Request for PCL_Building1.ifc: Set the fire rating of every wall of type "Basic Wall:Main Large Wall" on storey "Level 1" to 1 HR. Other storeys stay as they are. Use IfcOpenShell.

First a look at what the model holds.

```python
import ifcopenshell
import ifcopenshell.util.element

model = ifcopenshell.open("PCL_Building1.ifc")
print(model.schema)
storey = next(s for s in model.by_type("IfcBuildingStorey") if s.Name == "Level 1")
walls = [e for e in ifcopenshell.util.element.get_decomposition(storey) if e.is_a("IfcWall")]
seen = {}
for e in walls:
    element_type = ifcopenshell.util.element.get_type(e)
    key = (element_type.Name if element_type != e and element_type else None, ifcopenshell.util.element.get_pset(e, "Pset_WallCommon", "FireRating"))
    seen[key] = seen.get(key, 0) + 1
for (name, value), count in sorted(seen.items(), key=str):
    print(count, "x", name, "|", value)
```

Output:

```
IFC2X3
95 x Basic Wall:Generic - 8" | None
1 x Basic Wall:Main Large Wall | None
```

```python
import ifcopenshell
import ifcopenshell.api.pset
import ifcopenshell.util.element

model = ifcopenshell.open("PCL_Building1.ifc")

storey = next(s for s in model.by_type("IfcBuildingStorey") if s.Name == "Level 1")
walls = [e for e in ifcopenshell.util.element.get_decomposition(storey) if e.is_a("IfcWall")]

count = 0
for e in walls:
    element_type = ifcopenshell.util.element.get_type(e)
    if element_type in (None, e) or element_type.Name != "Basic Wall:Main Large Wall":
        continue
    # add_pset returns the element's existing set when there is one.
    pset = ifcopenshell.api.pset.add_pset(model, product=e, name="Pset_WallCommon")
    ifcopenshell.api.pset.edit_pset(model, pset=pset, properties={"FireRating": "1 HR"})
    count += 1

print(count, "walls updated")

model.write("PCL_Building1_edited.ifc")
```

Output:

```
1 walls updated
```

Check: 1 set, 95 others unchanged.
